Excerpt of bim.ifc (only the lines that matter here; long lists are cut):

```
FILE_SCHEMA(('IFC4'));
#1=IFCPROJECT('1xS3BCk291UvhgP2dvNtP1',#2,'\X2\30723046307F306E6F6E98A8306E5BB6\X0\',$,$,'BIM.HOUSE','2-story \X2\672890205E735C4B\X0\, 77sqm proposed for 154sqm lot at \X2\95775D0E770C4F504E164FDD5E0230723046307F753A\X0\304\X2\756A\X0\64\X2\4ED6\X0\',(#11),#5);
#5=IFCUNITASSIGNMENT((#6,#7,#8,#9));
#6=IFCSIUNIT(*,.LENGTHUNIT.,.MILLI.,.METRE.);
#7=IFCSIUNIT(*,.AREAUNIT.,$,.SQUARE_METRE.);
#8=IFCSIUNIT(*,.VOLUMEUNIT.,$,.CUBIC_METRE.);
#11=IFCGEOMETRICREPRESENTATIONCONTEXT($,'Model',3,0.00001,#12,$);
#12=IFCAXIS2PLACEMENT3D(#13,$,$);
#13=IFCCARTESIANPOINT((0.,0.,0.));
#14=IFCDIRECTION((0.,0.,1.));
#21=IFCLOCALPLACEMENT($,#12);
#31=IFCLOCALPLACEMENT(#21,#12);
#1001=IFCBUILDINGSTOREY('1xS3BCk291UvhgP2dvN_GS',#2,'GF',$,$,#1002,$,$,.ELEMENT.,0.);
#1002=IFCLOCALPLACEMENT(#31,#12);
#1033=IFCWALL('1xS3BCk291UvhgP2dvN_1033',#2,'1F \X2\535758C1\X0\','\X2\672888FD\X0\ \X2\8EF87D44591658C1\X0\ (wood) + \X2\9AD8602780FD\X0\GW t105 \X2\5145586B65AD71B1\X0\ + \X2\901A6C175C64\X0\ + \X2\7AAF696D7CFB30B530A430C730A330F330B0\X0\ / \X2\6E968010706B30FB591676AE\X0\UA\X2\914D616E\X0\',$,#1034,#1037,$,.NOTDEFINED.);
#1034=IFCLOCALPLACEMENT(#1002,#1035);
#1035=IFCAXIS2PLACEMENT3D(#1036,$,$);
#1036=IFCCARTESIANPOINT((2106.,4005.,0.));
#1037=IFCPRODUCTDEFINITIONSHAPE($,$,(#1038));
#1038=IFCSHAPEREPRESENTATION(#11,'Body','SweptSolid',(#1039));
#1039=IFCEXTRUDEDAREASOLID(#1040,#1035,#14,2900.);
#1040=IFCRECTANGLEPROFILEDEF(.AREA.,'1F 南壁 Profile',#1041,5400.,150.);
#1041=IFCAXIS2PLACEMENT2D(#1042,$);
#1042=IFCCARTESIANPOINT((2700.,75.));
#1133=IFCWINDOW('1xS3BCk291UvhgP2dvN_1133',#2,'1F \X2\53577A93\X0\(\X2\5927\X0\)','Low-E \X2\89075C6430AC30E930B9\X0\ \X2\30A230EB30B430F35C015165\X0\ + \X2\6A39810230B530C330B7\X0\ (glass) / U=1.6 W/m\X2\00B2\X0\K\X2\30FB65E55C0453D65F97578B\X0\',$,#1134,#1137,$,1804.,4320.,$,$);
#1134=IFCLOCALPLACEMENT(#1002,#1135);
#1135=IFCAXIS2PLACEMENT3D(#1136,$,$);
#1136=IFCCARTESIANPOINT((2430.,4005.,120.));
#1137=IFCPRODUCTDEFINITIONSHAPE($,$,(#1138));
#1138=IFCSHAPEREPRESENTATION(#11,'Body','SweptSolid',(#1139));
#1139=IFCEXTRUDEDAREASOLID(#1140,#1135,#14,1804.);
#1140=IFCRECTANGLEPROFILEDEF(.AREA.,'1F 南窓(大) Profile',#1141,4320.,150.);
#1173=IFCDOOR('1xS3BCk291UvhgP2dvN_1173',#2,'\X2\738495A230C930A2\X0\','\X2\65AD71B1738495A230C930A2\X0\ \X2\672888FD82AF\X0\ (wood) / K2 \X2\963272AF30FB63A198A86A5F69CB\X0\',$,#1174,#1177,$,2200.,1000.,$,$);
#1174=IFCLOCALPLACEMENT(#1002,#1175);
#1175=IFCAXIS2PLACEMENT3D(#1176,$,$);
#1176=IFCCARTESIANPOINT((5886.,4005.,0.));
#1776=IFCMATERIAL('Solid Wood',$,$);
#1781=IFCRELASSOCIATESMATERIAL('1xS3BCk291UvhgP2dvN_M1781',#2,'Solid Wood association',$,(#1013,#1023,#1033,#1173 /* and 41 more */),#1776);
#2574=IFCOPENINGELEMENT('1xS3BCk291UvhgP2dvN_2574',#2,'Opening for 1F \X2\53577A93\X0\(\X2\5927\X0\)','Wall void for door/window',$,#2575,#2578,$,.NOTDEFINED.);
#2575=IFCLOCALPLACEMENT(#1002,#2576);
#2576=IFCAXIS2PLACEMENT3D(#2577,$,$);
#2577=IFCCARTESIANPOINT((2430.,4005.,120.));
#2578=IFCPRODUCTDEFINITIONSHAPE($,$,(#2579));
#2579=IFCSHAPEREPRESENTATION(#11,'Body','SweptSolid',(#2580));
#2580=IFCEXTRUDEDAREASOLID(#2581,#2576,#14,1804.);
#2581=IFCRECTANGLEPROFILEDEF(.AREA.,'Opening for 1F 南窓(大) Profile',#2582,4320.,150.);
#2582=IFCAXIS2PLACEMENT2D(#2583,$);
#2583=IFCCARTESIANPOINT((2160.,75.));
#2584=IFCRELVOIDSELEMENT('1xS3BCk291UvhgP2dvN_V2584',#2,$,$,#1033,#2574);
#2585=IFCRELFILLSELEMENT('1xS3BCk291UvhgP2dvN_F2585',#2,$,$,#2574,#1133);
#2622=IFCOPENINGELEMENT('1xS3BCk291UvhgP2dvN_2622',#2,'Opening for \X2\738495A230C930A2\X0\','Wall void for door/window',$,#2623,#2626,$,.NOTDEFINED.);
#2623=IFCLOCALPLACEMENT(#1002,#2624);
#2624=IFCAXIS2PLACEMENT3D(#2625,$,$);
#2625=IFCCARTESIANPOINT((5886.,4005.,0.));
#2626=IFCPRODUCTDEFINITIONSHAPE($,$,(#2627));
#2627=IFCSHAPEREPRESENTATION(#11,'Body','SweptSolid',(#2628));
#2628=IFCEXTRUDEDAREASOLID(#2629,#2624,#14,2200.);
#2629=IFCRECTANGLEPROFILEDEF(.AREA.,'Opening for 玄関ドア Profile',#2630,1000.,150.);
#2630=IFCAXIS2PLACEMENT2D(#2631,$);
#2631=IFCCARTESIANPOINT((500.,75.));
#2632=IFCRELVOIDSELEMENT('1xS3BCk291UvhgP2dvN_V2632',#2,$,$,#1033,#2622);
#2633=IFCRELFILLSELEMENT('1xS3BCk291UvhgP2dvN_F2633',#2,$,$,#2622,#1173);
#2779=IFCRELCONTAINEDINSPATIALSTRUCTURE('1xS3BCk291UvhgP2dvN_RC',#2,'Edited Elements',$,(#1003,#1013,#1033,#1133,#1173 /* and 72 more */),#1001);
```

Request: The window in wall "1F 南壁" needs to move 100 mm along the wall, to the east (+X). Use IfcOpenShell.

```python
import ifcopenshell
import ifcopenshell.api.geometry
import ifcopenshell.util.placement

model = ifcopenshell.open("bim.ifc")

window = model.by_guid("1xS3BCk291UvhgP2dvN_1133")
opening = window.FillsVoids[0].RelatingOpeningElement
wall = opening.VoidsElements[0].RelatingBuildingElement

wall_matrix = ifcopenshell.util.placement.get_local_placement(wall.ObjectPlacement)
shift = wall_matrix[:3, 0] * 100.0
before = ifcopenshell.util.placement.get_local_placement(window.ObjectPlacement)[:3, 3].copy()

# The window is not placed relative to its opening, so move both.
for product in (opening, window):
    matrix = ifcopenshell.util.placement.get_local_placement(product.ObjectPlacement)
    matrix[:3, 3] += shift
    ifcopenshell.api.geometry.edit_object_placement(model, product=product, matrix=matrix, is_si=False)

after = ifcopenshell.util.placement.get_local_placement(window.ObjectPlacement)[:3, 3]
print("window moved by", (after - before).round(3) + 0.0)

model.write("bim-out.ifc")
```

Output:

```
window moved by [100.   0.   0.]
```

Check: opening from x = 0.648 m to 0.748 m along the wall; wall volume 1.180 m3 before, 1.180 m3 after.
